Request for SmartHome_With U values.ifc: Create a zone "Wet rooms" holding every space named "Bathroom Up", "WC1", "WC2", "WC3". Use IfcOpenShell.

First a look at what the model holds.

```python
import ifcopenshell

model = ifcopenshell.open("SmartHome_With U values.ifc")
print(model.schema)
seen = {}
for space in model.by_type("IfcSpace"):
    seen[space.LongName] = seen.get(space.LongName, 0) + 1
for name, count in sorted(seen.items(), key=str):
    print(count, "x", name)
print("zones:", [z.Name for z in model.by_type("IfcZone")][:20])
```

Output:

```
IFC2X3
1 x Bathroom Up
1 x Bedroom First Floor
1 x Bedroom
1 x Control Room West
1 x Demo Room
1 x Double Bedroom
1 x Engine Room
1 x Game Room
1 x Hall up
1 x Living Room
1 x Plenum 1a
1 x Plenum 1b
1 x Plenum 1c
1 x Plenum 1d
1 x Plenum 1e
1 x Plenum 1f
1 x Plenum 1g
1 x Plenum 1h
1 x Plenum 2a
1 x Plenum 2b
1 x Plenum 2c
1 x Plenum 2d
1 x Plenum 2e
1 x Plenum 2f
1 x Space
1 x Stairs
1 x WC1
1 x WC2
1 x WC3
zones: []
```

```python
import ifcopenshell
import ifcopenshell.api.group
import ifcopenshell.api.root

model = ifcopenshell.open("SmartHome_With U values.ifc")

names = {"Bathroom Up", "WC1", "WC2", "WC3"}
spaces = [s for s in model.by_type("IfcSpace") if s.LongName in names]

zone = ifcopenshell.api.root.create_entity(model, ifc_class="IfcZone", name="Wet rooms")
ifcopenshell.api.group.assign_group(model, products=spaces, group=zone)
print(len(spaces), "spaces in", zone.Name)

model.write("SmartHome_With U values_edited.ifc")
```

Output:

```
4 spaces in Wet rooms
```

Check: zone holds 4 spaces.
